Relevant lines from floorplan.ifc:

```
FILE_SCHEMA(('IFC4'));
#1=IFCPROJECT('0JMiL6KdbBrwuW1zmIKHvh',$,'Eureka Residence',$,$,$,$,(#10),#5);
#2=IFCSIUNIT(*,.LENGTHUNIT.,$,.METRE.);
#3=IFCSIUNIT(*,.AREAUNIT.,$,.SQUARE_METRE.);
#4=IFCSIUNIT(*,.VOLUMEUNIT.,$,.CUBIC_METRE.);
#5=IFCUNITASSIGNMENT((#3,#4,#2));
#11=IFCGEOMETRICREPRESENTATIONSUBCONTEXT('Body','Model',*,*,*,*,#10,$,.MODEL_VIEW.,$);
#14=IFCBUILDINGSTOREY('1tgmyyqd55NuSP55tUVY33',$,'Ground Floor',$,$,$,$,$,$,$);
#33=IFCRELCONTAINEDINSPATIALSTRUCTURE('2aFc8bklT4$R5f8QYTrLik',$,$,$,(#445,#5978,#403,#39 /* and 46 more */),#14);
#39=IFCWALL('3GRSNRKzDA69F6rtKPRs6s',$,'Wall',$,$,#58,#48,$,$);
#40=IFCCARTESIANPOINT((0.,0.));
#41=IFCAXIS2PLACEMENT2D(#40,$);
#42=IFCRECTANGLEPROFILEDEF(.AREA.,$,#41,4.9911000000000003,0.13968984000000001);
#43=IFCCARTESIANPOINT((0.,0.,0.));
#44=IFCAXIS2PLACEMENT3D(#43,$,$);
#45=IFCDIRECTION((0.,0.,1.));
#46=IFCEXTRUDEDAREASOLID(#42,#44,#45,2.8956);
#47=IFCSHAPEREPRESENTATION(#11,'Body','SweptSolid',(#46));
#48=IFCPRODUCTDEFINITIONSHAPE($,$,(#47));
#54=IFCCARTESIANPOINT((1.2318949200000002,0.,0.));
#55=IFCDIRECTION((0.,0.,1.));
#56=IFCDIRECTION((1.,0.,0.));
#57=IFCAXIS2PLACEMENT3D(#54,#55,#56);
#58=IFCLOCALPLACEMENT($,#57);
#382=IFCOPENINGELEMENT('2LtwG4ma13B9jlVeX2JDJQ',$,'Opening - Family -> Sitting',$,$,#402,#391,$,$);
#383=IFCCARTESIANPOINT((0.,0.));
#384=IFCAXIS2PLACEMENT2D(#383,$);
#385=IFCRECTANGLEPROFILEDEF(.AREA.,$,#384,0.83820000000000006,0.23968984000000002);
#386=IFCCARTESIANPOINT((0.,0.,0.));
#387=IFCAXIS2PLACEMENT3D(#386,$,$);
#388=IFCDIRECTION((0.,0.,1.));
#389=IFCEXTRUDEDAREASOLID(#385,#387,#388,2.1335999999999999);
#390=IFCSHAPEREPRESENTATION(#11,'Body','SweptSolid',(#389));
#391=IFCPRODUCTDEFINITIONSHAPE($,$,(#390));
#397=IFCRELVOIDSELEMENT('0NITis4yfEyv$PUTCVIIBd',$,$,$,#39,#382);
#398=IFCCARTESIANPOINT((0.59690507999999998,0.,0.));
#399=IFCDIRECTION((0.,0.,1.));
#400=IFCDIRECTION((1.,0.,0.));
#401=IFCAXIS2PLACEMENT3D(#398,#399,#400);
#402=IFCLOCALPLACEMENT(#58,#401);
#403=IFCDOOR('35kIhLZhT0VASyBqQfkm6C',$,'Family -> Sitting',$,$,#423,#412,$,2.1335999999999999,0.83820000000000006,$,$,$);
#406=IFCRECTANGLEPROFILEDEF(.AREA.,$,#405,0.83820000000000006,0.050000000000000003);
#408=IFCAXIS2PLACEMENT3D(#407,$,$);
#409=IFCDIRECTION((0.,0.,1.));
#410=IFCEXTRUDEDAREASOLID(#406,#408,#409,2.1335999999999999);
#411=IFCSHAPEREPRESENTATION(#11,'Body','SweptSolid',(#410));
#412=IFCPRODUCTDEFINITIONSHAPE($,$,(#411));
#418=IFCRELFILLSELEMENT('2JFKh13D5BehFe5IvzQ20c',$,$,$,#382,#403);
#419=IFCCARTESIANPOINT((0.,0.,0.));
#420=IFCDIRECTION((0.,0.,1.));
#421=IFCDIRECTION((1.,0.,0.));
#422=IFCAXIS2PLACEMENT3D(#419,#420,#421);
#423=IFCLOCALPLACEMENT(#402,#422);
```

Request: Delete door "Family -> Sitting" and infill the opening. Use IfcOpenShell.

```python
import ifcopenshell
import ifcopenshell.api.feature
import ifcopenshell.api.root
import ifcopenshell.geom
import ifcopenshell.util.shape

model = ifcopenshell.open("floorplan.ifc")
settings = ifcopenshell.geom.settings()


def volume(element):
    """Net volume in cubic metres, openings subtracted."""
    shape = ifcopenshell.geom.create_shape(settings, element)
    return ifcopenshell.util.shape.get_volume(shape.geometry)


door = model.by_guid("35kIhLZhT0VASyBqQfkm6C")
opening = door.FillsVoids[0].RelatingOpeningElement
wall = opening.VoidsElements[0].RelatingBuildingElement
before = volume(wall)

ifcopenshell.api.root.remove_product(model, product=door)
ifcopenshell.api.feature.remove_feature(model, feature=opening)

after = volume(wall)

print(f"wall volume {before:.3f} -> {after:.3f} m3")

model.write("floorplan_v2.ifc")
```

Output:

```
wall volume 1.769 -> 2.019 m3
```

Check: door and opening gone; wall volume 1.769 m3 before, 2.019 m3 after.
